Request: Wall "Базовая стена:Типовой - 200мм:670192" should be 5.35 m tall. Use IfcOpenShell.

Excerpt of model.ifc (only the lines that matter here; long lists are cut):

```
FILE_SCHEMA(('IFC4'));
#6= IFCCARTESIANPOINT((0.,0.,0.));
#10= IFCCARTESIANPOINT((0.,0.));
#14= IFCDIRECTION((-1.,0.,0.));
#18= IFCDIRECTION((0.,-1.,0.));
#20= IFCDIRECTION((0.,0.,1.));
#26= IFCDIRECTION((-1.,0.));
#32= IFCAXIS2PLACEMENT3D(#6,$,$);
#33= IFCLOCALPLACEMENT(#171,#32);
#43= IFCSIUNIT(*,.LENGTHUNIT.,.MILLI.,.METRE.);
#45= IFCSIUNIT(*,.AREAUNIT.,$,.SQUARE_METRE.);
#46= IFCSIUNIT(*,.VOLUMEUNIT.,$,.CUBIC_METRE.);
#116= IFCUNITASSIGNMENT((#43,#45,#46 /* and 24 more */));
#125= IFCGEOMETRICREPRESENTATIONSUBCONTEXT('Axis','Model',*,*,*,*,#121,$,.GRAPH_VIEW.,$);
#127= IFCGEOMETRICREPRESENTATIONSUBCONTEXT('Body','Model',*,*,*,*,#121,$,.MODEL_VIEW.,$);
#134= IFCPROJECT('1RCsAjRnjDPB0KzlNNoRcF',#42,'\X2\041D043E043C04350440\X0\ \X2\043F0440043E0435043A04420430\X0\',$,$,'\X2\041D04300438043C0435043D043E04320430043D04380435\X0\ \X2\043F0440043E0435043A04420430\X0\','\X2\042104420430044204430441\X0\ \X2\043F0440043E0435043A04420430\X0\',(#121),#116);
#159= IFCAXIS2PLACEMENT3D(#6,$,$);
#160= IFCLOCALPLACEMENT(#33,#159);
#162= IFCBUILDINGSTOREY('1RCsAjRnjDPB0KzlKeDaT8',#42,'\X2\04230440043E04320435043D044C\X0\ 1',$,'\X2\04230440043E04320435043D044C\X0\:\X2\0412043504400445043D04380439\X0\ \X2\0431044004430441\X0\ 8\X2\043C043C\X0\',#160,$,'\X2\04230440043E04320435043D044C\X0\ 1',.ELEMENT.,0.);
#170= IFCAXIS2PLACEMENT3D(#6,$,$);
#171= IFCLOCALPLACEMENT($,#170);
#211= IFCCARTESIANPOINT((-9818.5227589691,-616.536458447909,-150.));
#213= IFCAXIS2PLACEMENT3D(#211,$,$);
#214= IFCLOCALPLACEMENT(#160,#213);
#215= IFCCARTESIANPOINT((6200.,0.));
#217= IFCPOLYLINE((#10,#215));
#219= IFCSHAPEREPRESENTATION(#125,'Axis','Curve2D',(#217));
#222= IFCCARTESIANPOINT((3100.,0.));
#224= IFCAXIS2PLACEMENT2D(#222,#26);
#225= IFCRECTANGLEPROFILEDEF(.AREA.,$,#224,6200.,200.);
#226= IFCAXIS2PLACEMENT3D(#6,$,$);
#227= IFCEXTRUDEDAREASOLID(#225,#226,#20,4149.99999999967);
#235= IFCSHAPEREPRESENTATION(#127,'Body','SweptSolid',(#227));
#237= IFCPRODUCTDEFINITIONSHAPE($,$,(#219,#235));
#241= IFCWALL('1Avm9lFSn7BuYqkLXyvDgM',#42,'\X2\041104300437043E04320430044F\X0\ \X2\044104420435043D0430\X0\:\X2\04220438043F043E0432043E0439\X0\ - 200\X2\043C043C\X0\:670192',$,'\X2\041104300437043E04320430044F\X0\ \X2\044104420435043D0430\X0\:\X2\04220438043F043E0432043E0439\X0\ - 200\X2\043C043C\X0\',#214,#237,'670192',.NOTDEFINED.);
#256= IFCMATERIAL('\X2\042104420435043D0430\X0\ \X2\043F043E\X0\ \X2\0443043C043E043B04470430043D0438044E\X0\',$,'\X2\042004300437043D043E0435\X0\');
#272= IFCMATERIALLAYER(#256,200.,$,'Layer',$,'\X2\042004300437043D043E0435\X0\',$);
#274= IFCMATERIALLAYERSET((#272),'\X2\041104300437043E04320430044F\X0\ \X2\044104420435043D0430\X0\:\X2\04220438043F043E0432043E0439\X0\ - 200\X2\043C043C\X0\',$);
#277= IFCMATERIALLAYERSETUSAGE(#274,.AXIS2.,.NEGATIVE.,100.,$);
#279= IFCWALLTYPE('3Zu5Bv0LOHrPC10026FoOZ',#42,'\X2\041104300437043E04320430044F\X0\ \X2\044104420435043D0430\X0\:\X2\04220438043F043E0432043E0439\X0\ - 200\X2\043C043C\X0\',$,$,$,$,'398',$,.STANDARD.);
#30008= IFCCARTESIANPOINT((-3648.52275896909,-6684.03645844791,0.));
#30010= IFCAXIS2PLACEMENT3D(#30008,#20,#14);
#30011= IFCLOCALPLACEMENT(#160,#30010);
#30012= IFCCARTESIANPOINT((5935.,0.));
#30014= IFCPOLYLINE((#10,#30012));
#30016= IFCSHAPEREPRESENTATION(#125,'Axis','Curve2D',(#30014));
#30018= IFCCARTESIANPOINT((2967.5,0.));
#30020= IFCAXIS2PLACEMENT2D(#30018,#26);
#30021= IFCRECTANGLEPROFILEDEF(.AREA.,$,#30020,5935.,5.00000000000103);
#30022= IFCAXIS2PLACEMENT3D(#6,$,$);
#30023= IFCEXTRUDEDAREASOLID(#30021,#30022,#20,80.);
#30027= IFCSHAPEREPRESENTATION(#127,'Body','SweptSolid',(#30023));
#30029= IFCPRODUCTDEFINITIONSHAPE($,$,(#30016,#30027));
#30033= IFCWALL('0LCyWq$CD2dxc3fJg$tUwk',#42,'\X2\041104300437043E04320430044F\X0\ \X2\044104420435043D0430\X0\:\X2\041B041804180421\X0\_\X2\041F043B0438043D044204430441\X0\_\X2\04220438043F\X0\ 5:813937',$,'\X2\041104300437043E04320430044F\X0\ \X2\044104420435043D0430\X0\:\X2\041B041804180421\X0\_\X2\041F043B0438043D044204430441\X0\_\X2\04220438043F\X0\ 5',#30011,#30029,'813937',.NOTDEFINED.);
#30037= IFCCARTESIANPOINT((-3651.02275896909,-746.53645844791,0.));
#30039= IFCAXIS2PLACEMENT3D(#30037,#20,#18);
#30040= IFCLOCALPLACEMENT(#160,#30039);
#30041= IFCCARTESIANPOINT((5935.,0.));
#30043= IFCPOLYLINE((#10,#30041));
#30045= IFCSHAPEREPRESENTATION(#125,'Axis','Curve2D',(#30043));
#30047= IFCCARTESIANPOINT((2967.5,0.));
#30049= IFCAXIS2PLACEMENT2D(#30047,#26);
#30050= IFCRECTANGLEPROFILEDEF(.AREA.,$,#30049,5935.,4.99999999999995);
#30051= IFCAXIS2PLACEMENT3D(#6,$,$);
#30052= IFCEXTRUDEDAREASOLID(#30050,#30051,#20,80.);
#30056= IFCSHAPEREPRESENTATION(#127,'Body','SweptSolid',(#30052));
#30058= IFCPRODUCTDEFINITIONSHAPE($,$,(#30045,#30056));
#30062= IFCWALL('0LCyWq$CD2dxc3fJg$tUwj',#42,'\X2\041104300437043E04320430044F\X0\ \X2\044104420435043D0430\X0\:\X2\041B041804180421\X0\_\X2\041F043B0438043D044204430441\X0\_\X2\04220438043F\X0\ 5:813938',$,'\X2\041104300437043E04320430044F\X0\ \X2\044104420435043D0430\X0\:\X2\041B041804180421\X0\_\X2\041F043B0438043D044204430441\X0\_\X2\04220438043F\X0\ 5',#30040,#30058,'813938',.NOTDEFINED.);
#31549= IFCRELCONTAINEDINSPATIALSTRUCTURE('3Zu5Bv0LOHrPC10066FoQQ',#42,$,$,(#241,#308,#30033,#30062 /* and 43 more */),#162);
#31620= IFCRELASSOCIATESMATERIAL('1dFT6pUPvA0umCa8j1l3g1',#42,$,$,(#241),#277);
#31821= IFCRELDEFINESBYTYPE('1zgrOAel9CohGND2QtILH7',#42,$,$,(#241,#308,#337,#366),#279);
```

```python
import ifcopenshell
import ifcopenshell.geom
import ifcopenshell.util.representation
import ifcopenshell.util.shape
import ifcopenshell.util.unit

model = ifcopenshell.open("model.ifc")
unit_scale = ifcopenshell.util.unit.calculate_unit_scale(model)
settings = ifcopenshell.geom.settings()


def volume(element):
    """Net volume in cubic metres, openings subtracted."""
    shape = ifcopenshell.geom.create_shape(settings, element)
    return ifcopenshell.util.shape.get_volume(shape.geometry)


wall = model.by_guid("1Avm9lFSn7BuYqkLXyvDgM")
before = volume(wall)

body = ifcopenshell.util.representation.get_representation(wall, "Model", "Body")
solid = body.Items[0]
old_height = solid.Depth
solid.Depth = 5.35 / unit_scale
after = volume(wall)

print(f"height {old_height:g} -> {solid.Depth:g}, volume {before:.3f} -> {after:.3f} m3")

model.write("model_updated.ifc")
```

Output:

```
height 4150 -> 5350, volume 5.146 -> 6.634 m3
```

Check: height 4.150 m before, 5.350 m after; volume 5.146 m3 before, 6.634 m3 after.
